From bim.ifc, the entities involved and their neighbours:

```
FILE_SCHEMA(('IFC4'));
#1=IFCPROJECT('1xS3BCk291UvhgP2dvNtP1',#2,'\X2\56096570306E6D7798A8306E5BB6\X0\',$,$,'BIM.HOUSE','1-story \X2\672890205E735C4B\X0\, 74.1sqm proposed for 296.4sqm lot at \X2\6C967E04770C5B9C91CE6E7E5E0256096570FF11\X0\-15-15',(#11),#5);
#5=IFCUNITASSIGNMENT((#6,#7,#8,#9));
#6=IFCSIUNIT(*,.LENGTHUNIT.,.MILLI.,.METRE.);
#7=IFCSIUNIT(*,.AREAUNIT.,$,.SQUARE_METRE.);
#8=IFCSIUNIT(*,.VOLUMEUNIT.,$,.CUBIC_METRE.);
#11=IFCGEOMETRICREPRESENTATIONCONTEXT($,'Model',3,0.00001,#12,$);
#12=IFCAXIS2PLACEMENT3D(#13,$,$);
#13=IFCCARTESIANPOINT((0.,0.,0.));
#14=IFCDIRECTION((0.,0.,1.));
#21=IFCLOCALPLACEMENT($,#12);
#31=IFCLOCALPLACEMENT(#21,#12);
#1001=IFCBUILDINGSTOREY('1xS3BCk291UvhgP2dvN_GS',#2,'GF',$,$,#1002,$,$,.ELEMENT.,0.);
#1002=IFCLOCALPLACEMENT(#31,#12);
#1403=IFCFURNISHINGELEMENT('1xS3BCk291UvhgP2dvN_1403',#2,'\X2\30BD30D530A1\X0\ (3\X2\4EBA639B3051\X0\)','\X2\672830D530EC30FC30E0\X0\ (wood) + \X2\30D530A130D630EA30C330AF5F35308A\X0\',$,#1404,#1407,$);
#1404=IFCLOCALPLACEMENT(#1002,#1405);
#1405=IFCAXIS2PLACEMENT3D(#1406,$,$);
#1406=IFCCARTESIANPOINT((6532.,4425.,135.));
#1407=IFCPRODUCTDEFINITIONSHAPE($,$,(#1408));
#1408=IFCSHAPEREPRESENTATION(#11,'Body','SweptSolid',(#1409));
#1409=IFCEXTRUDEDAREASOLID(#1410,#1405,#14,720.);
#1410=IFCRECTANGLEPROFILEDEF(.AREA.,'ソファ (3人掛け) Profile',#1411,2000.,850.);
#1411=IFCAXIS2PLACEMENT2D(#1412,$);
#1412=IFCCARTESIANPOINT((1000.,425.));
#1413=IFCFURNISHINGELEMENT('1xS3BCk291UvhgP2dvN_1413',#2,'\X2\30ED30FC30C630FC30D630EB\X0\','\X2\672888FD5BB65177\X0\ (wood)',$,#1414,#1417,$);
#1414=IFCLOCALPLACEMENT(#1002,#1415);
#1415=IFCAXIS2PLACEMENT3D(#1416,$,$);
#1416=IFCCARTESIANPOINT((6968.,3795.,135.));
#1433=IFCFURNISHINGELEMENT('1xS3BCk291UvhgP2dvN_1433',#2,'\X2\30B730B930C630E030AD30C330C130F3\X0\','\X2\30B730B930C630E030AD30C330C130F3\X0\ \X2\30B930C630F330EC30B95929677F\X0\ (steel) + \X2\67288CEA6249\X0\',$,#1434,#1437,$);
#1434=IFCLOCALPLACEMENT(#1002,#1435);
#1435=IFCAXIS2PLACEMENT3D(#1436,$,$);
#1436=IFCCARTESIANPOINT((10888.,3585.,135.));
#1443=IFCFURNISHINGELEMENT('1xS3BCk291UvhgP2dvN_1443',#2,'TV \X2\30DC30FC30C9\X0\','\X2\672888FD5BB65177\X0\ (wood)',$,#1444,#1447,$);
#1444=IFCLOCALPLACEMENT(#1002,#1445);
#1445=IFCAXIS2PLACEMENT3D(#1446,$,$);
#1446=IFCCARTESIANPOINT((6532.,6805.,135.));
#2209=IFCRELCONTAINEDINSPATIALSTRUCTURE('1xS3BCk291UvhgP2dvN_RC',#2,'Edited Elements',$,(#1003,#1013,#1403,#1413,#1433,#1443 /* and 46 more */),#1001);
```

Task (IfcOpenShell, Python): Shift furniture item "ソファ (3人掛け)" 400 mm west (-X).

```python
import ifcopenshell
import ifcopenshell.api.geometry
import ifcopenshell.util.placement

model = ifcopenshell.open("bim.ifc")

item = model.by_guid("1xS3BCk291UvhgP2dvN_1403")
matrix = ifcopenshell.util.placement.get_local_placement(item.ObjectPlacement)
matrix[0, 3] -= 400.0
ifcopenshell.api.geometry.edit_object_placement(model, product=item, matrix=matrix, is_si=False)

print(ifcopenshell.util.placement.get_local_placement(item.ObjectPlacement).round(3) + 0.0)

model.write("bim-out.ifc")
```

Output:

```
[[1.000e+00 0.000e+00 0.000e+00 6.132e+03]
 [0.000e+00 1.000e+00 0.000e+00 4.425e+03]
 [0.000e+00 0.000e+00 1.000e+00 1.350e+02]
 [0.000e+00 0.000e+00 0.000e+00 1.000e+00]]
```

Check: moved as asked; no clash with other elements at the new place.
